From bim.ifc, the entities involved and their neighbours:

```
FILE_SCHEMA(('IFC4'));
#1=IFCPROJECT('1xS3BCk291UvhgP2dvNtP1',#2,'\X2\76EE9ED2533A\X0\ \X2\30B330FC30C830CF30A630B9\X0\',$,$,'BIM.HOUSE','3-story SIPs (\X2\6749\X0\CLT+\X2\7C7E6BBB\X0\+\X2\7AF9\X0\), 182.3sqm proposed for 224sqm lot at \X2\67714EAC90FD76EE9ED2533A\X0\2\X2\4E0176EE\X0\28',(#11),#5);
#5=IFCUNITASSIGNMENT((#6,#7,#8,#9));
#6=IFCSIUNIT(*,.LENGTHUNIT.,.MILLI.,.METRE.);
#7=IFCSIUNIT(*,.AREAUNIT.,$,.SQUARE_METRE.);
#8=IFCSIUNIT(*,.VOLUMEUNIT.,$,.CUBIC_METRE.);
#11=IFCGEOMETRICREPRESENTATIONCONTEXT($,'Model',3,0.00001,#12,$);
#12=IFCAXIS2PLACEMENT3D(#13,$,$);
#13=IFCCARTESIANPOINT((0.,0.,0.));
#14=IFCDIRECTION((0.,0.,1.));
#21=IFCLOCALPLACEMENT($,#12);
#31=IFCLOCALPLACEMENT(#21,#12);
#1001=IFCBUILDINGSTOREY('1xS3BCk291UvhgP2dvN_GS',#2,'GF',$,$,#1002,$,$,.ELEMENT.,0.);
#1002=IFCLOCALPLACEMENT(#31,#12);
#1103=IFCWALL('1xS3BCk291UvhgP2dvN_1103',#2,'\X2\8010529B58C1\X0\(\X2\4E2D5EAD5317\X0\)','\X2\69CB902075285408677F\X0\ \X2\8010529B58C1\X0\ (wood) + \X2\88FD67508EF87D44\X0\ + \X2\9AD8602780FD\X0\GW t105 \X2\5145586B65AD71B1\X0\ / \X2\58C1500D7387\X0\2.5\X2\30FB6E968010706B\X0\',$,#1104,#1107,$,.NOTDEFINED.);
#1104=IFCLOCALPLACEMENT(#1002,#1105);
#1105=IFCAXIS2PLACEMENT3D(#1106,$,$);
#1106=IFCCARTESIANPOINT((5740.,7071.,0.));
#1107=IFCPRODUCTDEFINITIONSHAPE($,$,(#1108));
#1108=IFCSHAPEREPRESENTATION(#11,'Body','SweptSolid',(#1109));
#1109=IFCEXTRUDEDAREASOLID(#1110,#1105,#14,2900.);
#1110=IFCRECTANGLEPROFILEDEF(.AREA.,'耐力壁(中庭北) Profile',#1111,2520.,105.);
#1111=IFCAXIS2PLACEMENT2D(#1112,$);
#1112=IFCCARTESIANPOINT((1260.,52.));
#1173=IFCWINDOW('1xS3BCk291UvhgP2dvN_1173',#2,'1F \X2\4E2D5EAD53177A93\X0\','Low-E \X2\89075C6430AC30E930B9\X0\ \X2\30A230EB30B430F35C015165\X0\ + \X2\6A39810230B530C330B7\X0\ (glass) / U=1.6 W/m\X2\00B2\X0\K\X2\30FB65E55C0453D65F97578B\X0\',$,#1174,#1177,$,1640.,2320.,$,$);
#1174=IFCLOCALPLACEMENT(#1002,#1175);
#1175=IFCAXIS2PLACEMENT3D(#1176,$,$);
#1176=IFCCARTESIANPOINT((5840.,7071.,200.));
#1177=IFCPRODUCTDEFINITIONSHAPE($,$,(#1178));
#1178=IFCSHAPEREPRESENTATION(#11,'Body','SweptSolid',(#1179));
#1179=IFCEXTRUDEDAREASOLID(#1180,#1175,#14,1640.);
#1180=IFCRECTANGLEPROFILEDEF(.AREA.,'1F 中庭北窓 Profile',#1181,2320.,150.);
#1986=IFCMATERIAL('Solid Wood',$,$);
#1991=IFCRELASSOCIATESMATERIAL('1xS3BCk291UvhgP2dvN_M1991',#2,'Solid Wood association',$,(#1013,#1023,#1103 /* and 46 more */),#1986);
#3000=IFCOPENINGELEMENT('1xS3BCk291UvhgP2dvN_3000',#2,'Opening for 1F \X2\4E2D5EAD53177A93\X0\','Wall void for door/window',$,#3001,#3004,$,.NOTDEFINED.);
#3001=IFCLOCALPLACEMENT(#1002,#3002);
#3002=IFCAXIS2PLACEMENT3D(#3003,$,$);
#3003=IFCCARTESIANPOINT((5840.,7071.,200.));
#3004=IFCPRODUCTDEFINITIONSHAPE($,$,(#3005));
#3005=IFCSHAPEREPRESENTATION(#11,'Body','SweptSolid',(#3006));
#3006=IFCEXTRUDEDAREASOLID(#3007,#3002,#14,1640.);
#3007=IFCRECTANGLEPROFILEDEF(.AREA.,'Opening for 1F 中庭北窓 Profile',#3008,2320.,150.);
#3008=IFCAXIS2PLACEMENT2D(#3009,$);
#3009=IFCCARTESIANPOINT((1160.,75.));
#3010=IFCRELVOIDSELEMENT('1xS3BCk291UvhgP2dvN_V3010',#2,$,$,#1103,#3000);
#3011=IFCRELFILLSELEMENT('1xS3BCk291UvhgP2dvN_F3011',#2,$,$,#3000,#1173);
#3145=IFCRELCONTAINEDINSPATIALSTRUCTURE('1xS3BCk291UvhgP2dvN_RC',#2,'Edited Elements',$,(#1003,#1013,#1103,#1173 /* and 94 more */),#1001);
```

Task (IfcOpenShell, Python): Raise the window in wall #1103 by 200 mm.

```python
import numpy as np
import ifcopenshell
import ifcopenshell.api.geometry
import ifcopenshell.util.placement
import ifcopenshell.util.unit

model = ifcopenshell.open("bim.ifc")
unit_scale = ifcopenshell.util.unit.calculate_unit_scale(model)

window = model.by_guid("1xS3BCk291UvhgP2dvN_1173")
opening = window.FillsVoids[0].RelatingOpeningElement
dz = 200.0

shift = np.array([0.0, 0.0, dz])
# The window is not placed relative to its opening, so move both.
for product in (opening, window):
    matrix = ifcopenshell.util.placement.get_local_placement(product.ObjectPlacement)
    matrix[:3, 3] += shift
    ifcopenshell.api.geometry.edit_object_placement(model, product=product, matrix=matrix, is_si=False)

print(f"moved by {dz * unit_scale:+.3f} m")

model.write("bim_rev.ifc")
```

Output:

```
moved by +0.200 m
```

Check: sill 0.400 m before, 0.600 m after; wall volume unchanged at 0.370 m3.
